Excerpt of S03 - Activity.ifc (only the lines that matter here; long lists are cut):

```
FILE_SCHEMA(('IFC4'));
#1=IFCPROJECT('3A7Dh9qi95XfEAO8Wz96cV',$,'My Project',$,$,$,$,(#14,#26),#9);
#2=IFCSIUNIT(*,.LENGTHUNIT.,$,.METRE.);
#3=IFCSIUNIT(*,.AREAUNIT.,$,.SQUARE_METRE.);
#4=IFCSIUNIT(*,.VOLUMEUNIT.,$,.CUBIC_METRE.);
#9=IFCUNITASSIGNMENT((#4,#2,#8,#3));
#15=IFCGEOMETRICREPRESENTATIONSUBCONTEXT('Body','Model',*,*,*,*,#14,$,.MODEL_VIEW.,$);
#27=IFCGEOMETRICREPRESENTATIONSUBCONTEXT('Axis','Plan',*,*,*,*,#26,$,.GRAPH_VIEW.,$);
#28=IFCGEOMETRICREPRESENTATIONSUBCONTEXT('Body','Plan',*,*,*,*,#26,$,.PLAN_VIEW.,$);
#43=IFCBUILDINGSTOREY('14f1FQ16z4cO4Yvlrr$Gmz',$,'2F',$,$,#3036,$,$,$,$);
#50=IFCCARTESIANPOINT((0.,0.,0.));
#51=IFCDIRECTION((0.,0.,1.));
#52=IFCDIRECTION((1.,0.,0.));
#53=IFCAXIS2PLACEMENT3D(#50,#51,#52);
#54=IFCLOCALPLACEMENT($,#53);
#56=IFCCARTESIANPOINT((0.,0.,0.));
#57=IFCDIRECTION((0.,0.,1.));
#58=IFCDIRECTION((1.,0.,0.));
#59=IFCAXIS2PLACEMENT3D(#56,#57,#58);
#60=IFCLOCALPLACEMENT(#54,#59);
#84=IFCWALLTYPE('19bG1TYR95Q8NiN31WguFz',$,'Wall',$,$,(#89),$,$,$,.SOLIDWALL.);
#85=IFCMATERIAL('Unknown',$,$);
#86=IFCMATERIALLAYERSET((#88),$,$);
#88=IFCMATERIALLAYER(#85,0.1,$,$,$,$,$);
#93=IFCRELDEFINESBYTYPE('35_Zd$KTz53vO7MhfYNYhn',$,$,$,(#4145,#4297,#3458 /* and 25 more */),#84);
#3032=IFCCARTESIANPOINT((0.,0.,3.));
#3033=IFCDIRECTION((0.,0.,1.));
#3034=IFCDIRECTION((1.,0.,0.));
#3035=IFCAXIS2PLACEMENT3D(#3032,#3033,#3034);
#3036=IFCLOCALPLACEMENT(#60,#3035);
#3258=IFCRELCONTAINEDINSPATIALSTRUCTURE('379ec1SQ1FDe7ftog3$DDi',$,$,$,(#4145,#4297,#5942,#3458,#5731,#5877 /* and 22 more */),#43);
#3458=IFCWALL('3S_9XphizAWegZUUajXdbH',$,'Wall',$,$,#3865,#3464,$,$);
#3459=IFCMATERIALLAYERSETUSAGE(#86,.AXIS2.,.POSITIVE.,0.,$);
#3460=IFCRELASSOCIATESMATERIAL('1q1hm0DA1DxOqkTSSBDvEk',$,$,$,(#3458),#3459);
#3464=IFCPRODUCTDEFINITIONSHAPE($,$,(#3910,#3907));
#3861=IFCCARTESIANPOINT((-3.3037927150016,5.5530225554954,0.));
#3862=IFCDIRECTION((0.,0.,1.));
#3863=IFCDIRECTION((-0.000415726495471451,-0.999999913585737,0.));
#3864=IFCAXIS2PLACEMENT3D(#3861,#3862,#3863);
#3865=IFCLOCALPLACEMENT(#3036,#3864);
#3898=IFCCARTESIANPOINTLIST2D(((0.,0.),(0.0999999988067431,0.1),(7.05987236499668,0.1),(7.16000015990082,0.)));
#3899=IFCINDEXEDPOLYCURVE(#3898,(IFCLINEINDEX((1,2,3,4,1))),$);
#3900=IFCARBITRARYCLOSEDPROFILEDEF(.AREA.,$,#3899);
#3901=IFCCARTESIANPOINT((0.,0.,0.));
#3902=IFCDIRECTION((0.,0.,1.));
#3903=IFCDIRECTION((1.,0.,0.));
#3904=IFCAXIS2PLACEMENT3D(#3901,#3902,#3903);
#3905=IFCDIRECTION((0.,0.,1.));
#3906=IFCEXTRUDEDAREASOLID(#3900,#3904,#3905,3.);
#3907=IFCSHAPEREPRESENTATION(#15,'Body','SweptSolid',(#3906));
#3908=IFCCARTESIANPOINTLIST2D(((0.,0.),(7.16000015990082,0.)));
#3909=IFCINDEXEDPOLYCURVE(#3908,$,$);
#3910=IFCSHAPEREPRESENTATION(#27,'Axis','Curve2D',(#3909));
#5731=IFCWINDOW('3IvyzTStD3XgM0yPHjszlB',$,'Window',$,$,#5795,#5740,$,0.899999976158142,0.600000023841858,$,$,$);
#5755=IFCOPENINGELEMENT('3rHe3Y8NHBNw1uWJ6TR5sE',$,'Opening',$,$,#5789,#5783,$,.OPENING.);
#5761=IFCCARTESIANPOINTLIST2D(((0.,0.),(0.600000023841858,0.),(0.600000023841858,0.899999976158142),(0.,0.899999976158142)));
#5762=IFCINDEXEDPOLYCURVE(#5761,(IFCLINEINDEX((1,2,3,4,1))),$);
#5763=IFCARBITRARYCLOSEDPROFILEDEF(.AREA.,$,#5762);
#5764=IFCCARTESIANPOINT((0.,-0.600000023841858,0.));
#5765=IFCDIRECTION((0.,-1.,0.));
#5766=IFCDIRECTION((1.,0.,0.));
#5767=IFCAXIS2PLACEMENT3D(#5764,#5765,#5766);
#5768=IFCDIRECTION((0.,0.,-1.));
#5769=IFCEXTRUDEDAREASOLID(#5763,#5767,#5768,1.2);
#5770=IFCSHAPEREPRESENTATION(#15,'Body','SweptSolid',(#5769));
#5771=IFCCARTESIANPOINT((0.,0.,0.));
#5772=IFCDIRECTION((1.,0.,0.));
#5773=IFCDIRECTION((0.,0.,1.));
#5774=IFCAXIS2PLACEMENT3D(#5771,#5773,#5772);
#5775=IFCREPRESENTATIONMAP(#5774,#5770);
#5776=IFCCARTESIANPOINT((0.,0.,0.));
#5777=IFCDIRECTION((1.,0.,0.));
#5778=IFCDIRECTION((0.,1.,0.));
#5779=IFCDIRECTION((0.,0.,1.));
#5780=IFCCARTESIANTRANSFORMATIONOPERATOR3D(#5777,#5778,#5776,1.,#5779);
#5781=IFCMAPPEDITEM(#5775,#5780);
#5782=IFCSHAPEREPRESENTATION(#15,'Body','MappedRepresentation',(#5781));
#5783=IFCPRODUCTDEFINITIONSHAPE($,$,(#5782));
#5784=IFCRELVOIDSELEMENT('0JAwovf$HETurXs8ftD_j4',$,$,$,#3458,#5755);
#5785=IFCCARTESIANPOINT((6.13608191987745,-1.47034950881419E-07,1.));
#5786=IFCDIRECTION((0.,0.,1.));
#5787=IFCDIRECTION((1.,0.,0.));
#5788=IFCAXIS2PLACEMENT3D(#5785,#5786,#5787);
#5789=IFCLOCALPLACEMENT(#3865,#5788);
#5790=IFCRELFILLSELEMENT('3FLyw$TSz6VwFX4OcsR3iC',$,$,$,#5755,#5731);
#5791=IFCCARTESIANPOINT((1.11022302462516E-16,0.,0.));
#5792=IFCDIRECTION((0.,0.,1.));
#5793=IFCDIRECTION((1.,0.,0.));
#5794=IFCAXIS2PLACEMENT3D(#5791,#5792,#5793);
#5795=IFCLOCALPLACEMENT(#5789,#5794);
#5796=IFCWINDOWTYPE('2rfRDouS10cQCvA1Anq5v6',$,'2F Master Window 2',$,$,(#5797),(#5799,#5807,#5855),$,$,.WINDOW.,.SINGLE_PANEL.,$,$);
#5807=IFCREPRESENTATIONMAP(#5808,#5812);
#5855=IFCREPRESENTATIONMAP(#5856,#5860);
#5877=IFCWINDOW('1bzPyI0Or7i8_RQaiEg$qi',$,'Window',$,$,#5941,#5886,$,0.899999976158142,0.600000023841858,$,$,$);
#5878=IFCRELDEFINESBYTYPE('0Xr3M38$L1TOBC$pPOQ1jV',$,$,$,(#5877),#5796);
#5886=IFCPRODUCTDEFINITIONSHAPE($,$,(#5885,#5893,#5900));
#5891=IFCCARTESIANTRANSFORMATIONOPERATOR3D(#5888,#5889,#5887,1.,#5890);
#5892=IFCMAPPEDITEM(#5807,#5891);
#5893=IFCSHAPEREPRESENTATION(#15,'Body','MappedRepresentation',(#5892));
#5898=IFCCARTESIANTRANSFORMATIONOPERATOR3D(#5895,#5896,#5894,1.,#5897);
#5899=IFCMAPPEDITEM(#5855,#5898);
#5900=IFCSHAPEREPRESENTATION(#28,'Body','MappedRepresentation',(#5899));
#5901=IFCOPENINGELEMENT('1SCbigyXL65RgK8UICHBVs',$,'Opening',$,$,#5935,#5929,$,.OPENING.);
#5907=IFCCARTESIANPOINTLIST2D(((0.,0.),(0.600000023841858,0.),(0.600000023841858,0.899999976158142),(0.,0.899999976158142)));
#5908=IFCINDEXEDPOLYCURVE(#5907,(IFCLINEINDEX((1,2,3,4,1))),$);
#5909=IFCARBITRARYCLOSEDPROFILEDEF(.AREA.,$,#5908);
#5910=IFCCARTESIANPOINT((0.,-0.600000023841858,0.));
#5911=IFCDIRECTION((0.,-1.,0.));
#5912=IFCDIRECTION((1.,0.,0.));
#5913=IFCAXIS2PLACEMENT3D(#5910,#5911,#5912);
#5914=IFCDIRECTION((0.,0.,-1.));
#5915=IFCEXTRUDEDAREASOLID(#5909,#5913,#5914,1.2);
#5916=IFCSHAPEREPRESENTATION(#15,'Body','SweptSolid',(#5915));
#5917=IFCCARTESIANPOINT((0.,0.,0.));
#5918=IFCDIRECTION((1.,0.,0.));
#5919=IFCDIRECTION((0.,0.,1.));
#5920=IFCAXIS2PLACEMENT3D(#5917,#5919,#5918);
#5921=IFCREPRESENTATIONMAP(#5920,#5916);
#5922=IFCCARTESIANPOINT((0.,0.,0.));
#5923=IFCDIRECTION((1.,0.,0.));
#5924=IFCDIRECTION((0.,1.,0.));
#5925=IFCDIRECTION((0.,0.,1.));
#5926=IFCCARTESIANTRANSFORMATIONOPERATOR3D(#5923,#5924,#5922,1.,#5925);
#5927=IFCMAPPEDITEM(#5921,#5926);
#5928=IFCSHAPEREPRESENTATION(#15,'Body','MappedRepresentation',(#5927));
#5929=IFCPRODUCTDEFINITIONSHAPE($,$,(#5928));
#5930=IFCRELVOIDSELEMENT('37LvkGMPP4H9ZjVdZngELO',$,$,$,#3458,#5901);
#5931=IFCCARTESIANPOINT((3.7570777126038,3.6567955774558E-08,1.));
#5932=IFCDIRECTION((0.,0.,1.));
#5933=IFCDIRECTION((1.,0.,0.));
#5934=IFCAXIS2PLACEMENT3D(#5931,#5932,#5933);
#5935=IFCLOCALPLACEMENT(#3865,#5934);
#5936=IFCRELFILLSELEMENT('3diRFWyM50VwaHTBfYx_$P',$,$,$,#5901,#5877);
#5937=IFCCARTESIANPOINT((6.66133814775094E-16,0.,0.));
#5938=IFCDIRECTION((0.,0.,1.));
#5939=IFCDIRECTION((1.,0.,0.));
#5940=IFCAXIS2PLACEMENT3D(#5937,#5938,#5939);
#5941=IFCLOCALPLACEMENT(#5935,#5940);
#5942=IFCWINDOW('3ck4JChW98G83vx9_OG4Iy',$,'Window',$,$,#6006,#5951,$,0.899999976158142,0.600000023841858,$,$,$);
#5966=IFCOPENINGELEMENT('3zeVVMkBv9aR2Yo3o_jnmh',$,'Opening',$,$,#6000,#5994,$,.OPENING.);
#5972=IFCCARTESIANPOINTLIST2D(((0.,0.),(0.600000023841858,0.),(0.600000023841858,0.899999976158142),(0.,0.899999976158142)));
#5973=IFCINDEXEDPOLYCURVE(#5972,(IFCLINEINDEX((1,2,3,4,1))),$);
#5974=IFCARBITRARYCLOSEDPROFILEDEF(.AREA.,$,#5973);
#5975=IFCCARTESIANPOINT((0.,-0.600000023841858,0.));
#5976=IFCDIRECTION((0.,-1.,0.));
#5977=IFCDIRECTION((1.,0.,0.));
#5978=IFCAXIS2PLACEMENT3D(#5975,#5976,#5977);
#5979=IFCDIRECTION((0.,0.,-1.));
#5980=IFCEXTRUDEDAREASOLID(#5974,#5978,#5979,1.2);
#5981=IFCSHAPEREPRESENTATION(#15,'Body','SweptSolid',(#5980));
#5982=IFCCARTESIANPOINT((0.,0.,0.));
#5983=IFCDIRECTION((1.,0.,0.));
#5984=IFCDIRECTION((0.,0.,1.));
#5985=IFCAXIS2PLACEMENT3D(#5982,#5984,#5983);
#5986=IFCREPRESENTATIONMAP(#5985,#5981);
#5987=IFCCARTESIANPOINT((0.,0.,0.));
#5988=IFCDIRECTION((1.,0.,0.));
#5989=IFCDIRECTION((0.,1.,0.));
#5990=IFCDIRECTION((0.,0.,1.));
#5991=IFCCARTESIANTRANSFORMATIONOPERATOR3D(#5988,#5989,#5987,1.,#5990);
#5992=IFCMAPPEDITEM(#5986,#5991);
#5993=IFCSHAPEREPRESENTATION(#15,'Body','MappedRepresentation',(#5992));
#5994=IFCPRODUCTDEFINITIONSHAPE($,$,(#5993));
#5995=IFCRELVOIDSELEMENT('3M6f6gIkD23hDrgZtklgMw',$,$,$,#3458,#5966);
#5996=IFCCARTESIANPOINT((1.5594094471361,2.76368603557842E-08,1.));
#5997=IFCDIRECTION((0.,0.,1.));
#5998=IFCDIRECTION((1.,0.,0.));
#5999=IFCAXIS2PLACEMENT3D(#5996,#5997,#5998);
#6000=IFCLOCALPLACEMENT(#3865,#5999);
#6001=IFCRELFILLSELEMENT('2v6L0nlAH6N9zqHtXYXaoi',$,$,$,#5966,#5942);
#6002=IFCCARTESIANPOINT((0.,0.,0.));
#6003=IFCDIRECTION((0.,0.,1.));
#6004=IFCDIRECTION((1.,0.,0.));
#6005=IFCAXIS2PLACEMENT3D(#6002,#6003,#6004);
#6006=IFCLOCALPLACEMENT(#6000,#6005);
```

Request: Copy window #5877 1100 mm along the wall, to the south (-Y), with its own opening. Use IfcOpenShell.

```python
import ifcopenshell
import ifcopenshell.api.feature
import ifcopenshell.api.geometry
import ifcopenshell.api.root
import ifcopenshell.geom
import ifcopenshell.util.element
import ifcopenshell.util.placement
import ifcopenshell.util.shape

model = ifcopenshell.open("S03 - Activity.ifc")
settings = ifcopenshell.geom.settings()


def volume(element):
    """Net volume in cubic metres, openings subtracted."""
    shape = ifcopenshell.geom.create_shape(settings, element)
    return ifcopenshell.util.shape.get_volume(shape.geometry)


window = model.by_guid("1bzPyI0Or7i8_RQaiEg$qi")
opening = window.FillsVoids[0].RelatingOpeningElement
wall = opening.VoidsElements[0].RelatingBuildingElement
before = volume(wall)
shift = ifcopenshell.util.placement.get_local_placement(wall.ObjectPlacement)[:3, 0] * 1.1

# copy_class copies the void relationship, type, container and properties, but no geometry.
new_opening = ifcopenshell.api.root.copy_class(model, product=opening)
new_opening.Representation = ifcopenshell.util.element.copy_deep(
    model, opening.Representation, exclude=["IfcGeometricRepresentationContext", "IfcRepresentationMap"]
)
new_window = ifcopenshell.api.root.copy_class(model, product=window)
new_window.Representation = ifcopenshell.util.element.copy_deep(
    model, window.Representation, exclude=["IfcGeometricRepresentationContext", "IfcRepresentationMap"]
)
ifcopenshell.api.feature.add_filling(model, opening=new_opening, element=new_window)

for old, new in ((opening, new_opening), (window, new_window)):
    matrix = ifcopenshell.util.placement.get_local_placement(old.ObjectPlacement)
    matrix[:3, 3] += shift
    ifcopenshell.api.geometry.edit_object_placement(model, product=new, matrix=matrix, is_si=False)

after = volume(wall)

print(f"wall volume {before:.3f} -> {after:.3f} m3")

model.write("S03 - Activity_rev.ifc")
```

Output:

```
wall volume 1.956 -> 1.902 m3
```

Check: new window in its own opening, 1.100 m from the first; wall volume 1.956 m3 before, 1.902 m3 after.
